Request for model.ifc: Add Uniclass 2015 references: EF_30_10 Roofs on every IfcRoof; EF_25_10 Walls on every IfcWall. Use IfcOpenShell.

First a look at what the model holds.

```python
import ifcopenshell

model = ifcopenshell.open("model.ifc")
print(model.schema)
print("classifications:", [c.Name for c in model.by_type("IfcClassification")])
for ifc_class in ("IfcDoor", "IfcRoof", "IfcStair", "IfcWall", "IfcWindow"):
    print(ifc_class, len(model.by_type(ifc_class)))
```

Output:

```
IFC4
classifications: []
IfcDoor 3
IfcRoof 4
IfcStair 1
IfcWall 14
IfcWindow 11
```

```python
import ifcopenshell
import ifcopenshell.api.classification

model = ifcopenshell.open("model.ifc")

system = ifcopenshell.api.classification.add_classification(model, classification="Uniclass 2015")

codes = {
    "IfcRoof": ("EF_30_10", "Roofs"),
    "IfcWall": ("EF_25_10", "Walls"),
}
for ifc_class, (code, name) in codes.items():
    products = model.by_type(ifc_class)
    ifcopenshell.api.classification.add_reference(
        model, products=products, classification=system, identification=code, name=name
    )
    print(code, len(products))

model.write("model_updated.ifc")
```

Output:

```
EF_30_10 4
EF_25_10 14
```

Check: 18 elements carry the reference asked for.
